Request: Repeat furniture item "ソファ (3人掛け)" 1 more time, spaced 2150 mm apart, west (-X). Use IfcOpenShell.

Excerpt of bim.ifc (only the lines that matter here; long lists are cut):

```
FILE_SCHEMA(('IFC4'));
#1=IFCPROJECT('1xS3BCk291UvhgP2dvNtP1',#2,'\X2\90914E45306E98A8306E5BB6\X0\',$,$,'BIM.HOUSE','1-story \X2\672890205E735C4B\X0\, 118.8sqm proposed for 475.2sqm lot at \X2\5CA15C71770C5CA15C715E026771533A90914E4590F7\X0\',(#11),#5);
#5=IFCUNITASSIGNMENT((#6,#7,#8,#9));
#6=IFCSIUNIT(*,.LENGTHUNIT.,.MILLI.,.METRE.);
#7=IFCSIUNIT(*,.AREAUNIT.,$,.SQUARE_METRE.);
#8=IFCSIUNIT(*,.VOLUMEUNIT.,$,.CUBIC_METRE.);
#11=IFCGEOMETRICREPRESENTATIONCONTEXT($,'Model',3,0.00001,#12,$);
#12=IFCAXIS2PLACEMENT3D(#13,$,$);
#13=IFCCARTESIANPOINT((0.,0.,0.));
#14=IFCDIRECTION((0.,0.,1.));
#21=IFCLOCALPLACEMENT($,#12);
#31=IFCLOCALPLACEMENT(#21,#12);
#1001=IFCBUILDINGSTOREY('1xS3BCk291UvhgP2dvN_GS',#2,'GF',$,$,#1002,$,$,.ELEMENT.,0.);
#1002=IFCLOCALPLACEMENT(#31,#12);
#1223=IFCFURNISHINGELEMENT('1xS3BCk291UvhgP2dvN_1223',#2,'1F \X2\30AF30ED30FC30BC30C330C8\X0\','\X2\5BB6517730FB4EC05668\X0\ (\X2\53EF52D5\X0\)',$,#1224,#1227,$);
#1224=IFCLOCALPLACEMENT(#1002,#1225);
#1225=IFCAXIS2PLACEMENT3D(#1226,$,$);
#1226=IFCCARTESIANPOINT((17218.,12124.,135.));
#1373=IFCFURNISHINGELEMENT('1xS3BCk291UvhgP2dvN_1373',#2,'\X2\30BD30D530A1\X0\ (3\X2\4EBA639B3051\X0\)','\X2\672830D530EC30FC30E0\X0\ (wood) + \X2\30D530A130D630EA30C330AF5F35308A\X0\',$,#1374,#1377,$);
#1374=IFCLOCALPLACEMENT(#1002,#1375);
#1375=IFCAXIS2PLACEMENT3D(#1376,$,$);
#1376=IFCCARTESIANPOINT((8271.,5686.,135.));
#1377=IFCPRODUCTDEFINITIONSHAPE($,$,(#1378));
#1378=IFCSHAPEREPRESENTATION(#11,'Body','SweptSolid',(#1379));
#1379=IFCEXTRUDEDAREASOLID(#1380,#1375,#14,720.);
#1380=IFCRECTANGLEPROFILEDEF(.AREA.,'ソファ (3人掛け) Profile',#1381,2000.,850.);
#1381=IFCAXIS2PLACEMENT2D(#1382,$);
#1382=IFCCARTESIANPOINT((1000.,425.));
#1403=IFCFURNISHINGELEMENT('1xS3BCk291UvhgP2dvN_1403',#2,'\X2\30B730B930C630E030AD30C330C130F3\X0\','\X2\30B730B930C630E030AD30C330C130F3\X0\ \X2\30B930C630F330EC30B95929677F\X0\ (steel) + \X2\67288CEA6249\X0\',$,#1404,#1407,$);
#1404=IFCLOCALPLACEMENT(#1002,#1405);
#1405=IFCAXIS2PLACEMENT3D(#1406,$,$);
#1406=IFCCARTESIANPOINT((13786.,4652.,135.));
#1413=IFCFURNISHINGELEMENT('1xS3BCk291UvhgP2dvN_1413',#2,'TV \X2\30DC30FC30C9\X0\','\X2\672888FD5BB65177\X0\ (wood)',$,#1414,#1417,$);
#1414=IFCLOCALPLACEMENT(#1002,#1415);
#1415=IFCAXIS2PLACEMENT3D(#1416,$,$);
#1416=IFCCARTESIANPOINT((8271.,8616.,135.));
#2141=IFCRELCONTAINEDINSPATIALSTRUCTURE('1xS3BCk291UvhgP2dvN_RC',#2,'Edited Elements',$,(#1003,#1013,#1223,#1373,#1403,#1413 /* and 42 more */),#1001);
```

```python
import numpy as np
import ifcopenshell
import ifcopenshell.api.geometry
import ifcopenshell.api.root
import ifcopenshell.util.element
import ifcopenshell.util.placement

model = ifcopenshell.open("bim.ifc")


def reuse_history(source, copy):
    """copy_class also copies each property set's owner history, people and application; keep the originals."""
    for rel in copy.IsDefinedBy:
        if rel.is_a("IfcRelDefinesByProperties") and (history := rel.RelatingPropertyDefinition.OwnerHistory):
            rel.RelatingPropertyDefinition.OwnerHistory = source.OwnerHistory
            ifcopenshell.util.element.remove_deep2(model, history)


source = model.by_id(1373)
base = ifcopenshell.util.placement.get_local_placement(source.ObjectPlacement)
step = np.array([-1.0, 0.0, 0.0]) * 2150.0

for i in range(1, 2):
    copy = ifcopenshell.api.root.copy_class(model, product=source)
    copy.Representation = ifcopenshell.util.element.copy_deep(
        model, source.Representation, exclude=["IfcGeometricRepresentationContext", "IfcRepresentationMap"]
    )
    reuse_history(source, copy)
    matrix = base.copy()
    matrix[:3, 3] += i * step
    print("added at", matrix[:3, 3].round(3) + 0.0)
    ifcopenshell.api.geometry.edit_object_placement(model, product=copy, matrix=matrix, is_si=False)

model.write("bim_edited.ifc")
```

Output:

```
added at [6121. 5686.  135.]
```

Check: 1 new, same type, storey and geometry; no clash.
